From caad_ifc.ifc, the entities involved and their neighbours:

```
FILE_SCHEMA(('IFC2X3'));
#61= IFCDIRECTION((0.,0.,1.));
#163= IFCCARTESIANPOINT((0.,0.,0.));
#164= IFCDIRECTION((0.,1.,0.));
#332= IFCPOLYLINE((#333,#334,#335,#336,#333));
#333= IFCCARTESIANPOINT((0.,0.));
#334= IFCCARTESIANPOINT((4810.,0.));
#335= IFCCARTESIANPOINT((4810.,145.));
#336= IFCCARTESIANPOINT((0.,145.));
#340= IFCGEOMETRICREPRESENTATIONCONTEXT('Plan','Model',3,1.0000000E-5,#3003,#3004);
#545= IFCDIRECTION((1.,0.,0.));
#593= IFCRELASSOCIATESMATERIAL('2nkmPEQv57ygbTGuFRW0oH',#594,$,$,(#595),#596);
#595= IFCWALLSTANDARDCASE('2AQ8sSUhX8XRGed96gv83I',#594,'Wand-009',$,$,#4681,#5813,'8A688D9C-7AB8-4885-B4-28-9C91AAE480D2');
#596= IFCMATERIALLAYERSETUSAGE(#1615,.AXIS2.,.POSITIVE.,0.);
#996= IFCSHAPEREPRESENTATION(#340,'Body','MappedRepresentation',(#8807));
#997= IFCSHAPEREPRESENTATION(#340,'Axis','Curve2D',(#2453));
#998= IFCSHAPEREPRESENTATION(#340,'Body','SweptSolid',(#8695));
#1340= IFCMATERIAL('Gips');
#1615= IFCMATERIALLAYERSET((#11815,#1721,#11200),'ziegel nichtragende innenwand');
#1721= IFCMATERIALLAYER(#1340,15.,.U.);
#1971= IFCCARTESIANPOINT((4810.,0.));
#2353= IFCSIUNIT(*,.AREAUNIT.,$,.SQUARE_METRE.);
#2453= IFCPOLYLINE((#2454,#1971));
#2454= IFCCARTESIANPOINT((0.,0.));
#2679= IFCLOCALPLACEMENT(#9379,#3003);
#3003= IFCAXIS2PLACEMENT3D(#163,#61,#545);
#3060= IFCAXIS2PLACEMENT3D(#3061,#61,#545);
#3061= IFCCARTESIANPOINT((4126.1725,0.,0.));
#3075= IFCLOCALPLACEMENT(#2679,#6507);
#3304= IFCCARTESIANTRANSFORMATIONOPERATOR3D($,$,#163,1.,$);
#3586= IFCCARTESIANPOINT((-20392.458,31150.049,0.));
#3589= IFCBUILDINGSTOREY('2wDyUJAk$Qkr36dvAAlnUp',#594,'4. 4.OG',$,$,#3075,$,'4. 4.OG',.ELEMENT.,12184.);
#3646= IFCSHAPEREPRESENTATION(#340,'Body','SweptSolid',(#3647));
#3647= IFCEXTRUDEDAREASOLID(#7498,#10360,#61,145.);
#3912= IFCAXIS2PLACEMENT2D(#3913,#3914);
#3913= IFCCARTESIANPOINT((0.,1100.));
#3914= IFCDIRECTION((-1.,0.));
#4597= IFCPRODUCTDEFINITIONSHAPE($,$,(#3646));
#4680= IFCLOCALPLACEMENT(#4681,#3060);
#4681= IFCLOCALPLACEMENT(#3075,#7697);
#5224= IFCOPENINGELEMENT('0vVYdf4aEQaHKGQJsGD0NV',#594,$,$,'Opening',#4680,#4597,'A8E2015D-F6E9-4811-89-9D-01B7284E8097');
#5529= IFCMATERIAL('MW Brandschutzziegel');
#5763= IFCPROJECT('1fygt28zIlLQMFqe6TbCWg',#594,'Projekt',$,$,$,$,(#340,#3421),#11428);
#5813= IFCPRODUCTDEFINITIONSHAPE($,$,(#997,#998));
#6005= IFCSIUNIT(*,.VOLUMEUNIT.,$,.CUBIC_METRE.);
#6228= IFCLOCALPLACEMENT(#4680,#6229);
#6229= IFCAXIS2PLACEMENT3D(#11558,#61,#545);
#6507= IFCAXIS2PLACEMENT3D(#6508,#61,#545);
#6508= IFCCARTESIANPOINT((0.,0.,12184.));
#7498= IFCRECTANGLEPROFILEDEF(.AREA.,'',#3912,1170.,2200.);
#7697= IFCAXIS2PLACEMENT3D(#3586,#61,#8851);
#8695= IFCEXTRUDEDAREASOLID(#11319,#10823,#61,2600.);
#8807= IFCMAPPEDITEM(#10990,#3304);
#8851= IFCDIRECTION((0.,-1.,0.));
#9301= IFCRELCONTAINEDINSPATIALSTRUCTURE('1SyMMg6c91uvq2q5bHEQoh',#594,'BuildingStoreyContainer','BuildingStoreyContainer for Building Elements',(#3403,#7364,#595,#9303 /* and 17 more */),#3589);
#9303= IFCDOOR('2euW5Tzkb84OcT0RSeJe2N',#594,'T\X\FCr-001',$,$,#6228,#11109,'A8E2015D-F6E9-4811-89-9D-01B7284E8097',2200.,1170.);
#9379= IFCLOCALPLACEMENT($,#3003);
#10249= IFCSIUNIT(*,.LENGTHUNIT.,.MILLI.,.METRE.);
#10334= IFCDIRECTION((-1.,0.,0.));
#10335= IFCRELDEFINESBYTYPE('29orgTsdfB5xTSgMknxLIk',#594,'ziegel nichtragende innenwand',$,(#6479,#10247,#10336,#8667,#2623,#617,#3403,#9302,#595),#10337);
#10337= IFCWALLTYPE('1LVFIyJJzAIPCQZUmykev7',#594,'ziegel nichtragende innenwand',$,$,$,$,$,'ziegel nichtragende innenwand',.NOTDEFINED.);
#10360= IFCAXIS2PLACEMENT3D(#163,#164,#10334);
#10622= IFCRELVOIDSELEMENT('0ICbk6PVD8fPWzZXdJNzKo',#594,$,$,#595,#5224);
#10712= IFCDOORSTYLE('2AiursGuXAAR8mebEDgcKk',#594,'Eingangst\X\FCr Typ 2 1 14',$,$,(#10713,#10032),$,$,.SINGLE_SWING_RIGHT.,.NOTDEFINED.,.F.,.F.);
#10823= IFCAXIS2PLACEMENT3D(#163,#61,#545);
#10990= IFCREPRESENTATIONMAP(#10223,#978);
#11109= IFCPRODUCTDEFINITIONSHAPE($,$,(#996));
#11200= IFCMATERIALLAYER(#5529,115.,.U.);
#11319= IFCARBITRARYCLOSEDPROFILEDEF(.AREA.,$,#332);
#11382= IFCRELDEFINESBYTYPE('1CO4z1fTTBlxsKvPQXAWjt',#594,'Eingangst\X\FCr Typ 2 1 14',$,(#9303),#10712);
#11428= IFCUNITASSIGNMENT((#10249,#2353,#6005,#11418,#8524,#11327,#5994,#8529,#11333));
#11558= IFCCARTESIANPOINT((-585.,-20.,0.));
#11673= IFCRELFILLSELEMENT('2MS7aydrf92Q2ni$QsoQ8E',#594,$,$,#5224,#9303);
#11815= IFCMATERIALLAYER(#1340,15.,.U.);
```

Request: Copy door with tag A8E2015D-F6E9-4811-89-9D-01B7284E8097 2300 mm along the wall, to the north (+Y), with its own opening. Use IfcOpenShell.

```python
import ifcopenshell
import ifcopenshell.api.feature
import ifcopenshell.api.geometry
import ifcopenshell.api.root
import ifcopenshell.geom
import ifcopenshell.util.element
import ifcopenshell.util.placement
import ifcopenshell.util.shape
import ifcopenshell.util.unit

model = ifcopenshell.open("caad_ifc.ifc")
unit_scale = ifcopenshell.util.unit.calculate_unit_scale(model)
settings = ifcopenshell.geom.settings()


def volume(element):
    """Net volume in cubic metres, openings subtracted."""
    shape = ifcopenshell.geom.create_shape(settings, element)
    return ifcopenshell.util.shape.get_volume(shape.geometry)


door = model.by_guid("2euW5Tzkb84OcT0RSeJe2N")
opening = door.FillsVoids[0].RelatingOpeningElement
wall = opening.VoidsElements[0].RelatingBuildingElement
before = volume(wall)
shift = ifcopenshell.util.placement.get_local_placement(wall.ObjectPlacement)[:3, 0] * -2.3 / unit_scale

# copy_class copies the void relationship, type, container and properties, but no geometry.
new_opening = ifcopenshell.api.root.copy_class(model, product=opening)
new_opening.Representation = ifcopenshell.util.element.copy_deep(
    model, opening.Representation, exclude=["IfcGeometricRepresentationContext", "IfcRepresentationMap"]
)
new_opening.Tag = None
new_door = ifcopenshell.api.root.copy_class(model, product=door)
new_door.Representation = ifcopenshell.util.element.copy_deep(
    model, door.Representation, exclude=["IfcGeometricRepresentationContext", "IfcRepresentationMap"]
)
new_door.Tag = None
fills = ifcopenshell.api.feature.add_filling(model, opening=new_opening, element=new_door)
fills.OwnerHistory = new_door.OwnerHistory  # required in IFC2X3

for old, new in ((opening, new_opening), (door, new_door)):
    matrix = ifcopenshell.util.placement.get_local_placement(old.ObjectPlacement)
    matrix[:3, 3] += shift
    ifcopenshell.api.geometry.edit_object_placement(model, product=new, matrix=matrix, is_si=False)

after = volume(wall)

print(f"wall volume {before:.3f} -> {after:.3f} m3")

model.write("caad_ifc_updated.ifc")
```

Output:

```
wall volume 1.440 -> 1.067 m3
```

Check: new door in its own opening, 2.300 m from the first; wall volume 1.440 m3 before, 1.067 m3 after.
